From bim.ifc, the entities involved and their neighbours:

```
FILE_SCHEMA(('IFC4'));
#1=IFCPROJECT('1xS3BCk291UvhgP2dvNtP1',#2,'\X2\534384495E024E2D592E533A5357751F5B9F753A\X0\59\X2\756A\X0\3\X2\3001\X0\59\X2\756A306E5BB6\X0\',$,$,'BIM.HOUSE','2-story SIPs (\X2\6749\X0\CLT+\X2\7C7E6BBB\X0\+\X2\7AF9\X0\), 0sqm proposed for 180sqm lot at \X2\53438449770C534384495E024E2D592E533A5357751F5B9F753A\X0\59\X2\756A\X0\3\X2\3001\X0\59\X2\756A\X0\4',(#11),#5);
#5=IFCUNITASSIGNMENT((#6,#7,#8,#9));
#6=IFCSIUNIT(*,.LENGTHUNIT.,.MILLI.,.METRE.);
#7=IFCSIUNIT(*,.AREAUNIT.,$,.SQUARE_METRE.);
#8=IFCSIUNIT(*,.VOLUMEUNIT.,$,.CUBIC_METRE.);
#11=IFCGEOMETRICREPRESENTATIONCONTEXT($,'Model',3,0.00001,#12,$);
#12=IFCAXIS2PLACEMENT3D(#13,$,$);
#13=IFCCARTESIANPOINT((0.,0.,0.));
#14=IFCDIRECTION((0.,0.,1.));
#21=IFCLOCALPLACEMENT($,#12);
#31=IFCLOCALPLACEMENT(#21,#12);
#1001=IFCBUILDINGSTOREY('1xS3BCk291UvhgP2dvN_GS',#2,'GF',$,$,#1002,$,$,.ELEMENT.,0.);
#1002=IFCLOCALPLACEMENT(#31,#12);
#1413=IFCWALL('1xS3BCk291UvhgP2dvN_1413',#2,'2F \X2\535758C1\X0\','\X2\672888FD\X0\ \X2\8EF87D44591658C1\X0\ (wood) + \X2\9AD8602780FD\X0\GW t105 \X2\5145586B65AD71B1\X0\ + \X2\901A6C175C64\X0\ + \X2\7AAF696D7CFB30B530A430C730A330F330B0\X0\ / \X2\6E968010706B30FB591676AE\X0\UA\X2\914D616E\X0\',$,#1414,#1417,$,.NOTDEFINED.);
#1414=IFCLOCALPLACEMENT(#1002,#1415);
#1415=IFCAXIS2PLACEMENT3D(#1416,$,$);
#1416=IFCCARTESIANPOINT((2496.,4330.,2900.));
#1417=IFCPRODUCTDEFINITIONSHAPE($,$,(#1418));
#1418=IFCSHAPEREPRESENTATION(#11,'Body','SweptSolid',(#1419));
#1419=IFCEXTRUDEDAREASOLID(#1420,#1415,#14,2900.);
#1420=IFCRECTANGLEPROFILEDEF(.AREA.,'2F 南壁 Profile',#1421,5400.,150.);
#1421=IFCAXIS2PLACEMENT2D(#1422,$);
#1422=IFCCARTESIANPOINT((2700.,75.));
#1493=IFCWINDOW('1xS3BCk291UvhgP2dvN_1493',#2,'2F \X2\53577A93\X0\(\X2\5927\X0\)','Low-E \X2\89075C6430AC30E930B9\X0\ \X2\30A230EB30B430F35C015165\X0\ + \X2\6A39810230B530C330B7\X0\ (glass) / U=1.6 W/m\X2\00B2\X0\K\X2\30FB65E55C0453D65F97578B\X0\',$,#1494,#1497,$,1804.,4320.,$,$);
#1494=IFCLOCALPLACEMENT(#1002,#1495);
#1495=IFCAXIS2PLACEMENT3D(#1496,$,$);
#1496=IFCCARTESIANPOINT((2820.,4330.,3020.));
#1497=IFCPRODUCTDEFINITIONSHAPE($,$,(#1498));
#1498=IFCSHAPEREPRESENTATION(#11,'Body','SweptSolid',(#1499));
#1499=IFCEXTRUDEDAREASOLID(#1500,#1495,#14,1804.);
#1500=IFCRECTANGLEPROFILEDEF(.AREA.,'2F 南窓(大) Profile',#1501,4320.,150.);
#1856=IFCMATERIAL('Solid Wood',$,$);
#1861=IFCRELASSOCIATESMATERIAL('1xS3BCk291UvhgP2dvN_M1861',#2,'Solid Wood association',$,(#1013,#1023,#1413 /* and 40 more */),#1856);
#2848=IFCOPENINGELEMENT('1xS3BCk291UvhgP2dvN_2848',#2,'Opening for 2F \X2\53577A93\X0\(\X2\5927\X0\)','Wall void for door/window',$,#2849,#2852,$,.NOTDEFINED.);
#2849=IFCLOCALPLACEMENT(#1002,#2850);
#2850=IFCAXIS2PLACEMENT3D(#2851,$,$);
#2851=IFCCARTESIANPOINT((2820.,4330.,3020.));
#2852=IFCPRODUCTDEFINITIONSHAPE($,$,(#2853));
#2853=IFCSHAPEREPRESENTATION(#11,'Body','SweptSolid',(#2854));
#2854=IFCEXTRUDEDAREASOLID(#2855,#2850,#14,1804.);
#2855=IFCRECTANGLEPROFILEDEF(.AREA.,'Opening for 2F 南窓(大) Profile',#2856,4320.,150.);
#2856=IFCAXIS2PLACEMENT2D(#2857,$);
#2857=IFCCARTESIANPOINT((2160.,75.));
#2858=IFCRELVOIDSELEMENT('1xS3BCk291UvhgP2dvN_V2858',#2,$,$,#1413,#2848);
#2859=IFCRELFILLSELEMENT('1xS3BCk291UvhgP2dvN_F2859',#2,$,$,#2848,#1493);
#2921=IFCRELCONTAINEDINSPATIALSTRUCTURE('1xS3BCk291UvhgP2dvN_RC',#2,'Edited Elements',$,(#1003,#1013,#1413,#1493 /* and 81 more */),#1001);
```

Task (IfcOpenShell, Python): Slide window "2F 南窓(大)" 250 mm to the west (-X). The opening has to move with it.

```python
import ifcopenshell
import ifcopenshell.api.geometry
import ifcopenshell.util.placement
import ifcopenshell.util.unit

model = ifcopenshell.open("bim.ifc")
unit_scale = ifcopenshell.util.unit.calculate_unit_scale(model)

window = model.by_guid("1xS3BCk291UvhgP2dvN_1493")
opening = window.FillsVoids[0].RelatingOpeningElement
wall = opening.VoidsElements[0].RelatingBuildingElement

wall_matrix = ifcopenshell.util.placement.get_local_placement(wall.ObjectPlacement)
shift = wall_matrix[:3, 0] * -0.25 / unit_scale
before = ifcopenshell.util.placement.get_local_placement(window.ObjectPlacement)[:3, 3].copy()

# The window is not placed relative to its opening, so move both.
for product in (opening, window):
    matrix = ifcopenshell.util.placement.get_local_placement(product.ObjectPlacement)
    matrix[:3, 3] += shift
    ifcopenshell.api.geometry.edit_object_placement(model, product=product, matrix=matrix, is_si=False)

after = ifcopenshell.util.placement.get_local_placement(window.ObjectPlacement)[:3, 3]
print("window moved by", (after - before).round(3) + 0.0)

model.write("bim_updated.ifc")
```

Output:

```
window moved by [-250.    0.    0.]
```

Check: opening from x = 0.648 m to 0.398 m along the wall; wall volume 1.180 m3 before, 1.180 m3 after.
